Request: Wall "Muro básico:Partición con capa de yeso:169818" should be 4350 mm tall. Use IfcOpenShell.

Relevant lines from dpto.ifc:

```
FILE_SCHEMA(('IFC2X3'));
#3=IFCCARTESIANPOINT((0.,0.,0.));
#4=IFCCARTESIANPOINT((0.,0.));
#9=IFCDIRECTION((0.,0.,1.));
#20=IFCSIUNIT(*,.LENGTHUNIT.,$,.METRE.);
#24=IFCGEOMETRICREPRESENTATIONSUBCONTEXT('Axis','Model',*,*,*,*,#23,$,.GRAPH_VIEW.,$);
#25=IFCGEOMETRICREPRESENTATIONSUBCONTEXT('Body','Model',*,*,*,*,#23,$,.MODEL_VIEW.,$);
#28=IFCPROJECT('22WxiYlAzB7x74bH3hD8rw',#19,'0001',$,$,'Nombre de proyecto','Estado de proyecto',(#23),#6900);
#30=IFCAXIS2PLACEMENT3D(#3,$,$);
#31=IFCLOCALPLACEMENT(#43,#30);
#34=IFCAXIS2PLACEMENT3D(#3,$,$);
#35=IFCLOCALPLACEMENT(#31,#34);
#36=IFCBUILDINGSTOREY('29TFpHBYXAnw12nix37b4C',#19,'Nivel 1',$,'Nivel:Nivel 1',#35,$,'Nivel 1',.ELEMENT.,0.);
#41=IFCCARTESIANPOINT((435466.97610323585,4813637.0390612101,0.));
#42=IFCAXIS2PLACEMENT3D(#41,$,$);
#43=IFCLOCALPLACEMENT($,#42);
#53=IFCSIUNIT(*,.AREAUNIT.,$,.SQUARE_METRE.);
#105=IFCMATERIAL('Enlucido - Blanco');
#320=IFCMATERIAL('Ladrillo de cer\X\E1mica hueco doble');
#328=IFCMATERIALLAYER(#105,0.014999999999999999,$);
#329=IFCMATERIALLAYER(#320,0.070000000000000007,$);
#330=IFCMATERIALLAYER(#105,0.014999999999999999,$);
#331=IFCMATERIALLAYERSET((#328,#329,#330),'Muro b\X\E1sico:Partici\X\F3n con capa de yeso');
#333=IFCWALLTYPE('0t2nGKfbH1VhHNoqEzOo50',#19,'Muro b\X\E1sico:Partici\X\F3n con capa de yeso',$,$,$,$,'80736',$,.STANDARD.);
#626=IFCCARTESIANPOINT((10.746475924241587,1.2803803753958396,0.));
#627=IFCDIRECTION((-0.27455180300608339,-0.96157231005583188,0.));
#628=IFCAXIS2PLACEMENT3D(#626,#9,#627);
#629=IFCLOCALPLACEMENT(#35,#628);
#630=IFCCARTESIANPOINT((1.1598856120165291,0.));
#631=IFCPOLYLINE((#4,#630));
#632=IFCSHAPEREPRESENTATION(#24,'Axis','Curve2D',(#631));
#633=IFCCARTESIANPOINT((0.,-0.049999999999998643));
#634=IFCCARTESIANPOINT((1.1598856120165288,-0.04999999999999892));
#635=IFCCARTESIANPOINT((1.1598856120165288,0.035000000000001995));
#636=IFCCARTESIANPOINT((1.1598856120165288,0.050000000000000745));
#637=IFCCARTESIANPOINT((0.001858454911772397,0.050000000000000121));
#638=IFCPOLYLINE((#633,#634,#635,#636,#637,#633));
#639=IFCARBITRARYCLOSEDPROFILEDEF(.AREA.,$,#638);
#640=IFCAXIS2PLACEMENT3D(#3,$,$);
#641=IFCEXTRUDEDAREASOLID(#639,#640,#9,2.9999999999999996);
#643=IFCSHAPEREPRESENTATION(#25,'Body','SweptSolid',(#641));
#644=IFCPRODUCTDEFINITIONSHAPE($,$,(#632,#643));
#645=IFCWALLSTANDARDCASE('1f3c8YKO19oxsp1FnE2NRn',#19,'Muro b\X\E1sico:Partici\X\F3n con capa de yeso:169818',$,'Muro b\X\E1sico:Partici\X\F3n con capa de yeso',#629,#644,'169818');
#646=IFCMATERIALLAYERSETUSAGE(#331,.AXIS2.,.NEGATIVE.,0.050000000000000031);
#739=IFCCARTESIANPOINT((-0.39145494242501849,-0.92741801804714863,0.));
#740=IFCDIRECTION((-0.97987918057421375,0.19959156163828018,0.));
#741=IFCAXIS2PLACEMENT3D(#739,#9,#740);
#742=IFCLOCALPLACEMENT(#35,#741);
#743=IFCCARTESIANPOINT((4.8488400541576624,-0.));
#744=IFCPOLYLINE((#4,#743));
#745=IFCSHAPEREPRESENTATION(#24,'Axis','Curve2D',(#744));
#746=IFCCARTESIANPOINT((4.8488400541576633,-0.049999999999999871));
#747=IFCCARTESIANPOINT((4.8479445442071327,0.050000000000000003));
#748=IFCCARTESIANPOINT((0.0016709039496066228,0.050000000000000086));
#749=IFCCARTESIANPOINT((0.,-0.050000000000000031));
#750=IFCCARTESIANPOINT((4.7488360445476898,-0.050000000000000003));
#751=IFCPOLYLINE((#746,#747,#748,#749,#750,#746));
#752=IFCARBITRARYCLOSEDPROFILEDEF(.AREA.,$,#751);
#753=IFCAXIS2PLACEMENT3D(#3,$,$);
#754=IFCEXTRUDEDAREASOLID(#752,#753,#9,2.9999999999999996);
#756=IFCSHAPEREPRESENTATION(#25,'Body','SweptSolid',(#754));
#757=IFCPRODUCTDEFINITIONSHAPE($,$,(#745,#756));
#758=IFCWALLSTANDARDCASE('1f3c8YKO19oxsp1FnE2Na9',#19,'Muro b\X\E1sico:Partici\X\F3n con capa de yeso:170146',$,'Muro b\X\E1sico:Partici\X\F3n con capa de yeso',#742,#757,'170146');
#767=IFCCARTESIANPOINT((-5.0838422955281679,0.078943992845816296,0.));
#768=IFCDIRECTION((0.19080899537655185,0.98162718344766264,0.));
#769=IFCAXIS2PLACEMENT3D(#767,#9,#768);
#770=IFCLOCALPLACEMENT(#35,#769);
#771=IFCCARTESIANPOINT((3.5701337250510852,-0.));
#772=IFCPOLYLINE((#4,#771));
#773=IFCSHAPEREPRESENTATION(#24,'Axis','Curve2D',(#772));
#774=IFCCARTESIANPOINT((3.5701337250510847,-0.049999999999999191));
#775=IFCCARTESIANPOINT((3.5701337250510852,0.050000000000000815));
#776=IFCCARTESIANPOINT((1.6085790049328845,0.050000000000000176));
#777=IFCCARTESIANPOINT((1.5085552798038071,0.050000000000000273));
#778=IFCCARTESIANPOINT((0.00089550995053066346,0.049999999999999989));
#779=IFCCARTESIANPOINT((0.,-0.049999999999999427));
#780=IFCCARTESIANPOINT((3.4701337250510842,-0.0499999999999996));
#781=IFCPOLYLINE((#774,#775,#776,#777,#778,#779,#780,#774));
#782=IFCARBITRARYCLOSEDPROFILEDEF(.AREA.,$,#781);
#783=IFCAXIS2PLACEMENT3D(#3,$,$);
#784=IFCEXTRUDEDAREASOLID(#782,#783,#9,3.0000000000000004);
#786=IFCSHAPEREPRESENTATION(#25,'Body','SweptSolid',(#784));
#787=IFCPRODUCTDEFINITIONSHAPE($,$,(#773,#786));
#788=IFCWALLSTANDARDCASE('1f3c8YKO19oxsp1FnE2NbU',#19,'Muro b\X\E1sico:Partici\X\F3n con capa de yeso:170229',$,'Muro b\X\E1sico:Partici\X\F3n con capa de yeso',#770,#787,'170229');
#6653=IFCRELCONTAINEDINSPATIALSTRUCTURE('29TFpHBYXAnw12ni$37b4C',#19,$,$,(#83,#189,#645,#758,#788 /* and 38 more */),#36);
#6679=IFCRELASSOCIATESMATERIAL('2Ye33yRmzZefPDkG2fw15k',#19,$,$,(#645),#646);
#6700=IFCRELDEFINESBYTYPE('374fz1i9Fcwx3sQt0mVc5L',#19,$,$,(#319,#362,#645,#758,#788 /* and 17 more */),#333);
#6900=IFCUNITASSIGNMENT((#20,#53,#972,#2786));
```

```python
import ifcopenshell
import ifcopenshell.geom
import ifcopenshell.util.representation
import ifcopenshell.util.shape
import ifcopenshell.util.unit

model = ifcopenshell.open("dpto.ifc")
unit_scale = ifcopenshell.util.unit.calculate_unit_scale(model)
settings = ifcopenshell.geom.settings()


def volume(element):
    """Net volume in cubic metres, openings subtracted."""
    shape = ifcopenshell.geom.create_shape(settings, element)
    return ifcopenshell.util.shape.get_volume(shape.geometry)


wall = model.by_id(645)
before = volume(wall)

body = ifcopenshell.util.representation.get_representation(wall, "Model", "Body")
solid = body.Items[0]
old_height = solid.Depth
solid.Depth = 4.35 / unit_scale
after = volume(wall)

print(f"height {old_height:g} -> {solid.Depth:g}, volume {before:.3f} -> {after:.3f} m3")

model.write("dpto_rev.ifc")
```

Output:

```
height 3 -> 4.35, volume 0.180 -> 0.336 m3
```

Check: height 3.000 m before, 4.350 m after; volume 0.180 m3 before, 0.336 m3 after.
